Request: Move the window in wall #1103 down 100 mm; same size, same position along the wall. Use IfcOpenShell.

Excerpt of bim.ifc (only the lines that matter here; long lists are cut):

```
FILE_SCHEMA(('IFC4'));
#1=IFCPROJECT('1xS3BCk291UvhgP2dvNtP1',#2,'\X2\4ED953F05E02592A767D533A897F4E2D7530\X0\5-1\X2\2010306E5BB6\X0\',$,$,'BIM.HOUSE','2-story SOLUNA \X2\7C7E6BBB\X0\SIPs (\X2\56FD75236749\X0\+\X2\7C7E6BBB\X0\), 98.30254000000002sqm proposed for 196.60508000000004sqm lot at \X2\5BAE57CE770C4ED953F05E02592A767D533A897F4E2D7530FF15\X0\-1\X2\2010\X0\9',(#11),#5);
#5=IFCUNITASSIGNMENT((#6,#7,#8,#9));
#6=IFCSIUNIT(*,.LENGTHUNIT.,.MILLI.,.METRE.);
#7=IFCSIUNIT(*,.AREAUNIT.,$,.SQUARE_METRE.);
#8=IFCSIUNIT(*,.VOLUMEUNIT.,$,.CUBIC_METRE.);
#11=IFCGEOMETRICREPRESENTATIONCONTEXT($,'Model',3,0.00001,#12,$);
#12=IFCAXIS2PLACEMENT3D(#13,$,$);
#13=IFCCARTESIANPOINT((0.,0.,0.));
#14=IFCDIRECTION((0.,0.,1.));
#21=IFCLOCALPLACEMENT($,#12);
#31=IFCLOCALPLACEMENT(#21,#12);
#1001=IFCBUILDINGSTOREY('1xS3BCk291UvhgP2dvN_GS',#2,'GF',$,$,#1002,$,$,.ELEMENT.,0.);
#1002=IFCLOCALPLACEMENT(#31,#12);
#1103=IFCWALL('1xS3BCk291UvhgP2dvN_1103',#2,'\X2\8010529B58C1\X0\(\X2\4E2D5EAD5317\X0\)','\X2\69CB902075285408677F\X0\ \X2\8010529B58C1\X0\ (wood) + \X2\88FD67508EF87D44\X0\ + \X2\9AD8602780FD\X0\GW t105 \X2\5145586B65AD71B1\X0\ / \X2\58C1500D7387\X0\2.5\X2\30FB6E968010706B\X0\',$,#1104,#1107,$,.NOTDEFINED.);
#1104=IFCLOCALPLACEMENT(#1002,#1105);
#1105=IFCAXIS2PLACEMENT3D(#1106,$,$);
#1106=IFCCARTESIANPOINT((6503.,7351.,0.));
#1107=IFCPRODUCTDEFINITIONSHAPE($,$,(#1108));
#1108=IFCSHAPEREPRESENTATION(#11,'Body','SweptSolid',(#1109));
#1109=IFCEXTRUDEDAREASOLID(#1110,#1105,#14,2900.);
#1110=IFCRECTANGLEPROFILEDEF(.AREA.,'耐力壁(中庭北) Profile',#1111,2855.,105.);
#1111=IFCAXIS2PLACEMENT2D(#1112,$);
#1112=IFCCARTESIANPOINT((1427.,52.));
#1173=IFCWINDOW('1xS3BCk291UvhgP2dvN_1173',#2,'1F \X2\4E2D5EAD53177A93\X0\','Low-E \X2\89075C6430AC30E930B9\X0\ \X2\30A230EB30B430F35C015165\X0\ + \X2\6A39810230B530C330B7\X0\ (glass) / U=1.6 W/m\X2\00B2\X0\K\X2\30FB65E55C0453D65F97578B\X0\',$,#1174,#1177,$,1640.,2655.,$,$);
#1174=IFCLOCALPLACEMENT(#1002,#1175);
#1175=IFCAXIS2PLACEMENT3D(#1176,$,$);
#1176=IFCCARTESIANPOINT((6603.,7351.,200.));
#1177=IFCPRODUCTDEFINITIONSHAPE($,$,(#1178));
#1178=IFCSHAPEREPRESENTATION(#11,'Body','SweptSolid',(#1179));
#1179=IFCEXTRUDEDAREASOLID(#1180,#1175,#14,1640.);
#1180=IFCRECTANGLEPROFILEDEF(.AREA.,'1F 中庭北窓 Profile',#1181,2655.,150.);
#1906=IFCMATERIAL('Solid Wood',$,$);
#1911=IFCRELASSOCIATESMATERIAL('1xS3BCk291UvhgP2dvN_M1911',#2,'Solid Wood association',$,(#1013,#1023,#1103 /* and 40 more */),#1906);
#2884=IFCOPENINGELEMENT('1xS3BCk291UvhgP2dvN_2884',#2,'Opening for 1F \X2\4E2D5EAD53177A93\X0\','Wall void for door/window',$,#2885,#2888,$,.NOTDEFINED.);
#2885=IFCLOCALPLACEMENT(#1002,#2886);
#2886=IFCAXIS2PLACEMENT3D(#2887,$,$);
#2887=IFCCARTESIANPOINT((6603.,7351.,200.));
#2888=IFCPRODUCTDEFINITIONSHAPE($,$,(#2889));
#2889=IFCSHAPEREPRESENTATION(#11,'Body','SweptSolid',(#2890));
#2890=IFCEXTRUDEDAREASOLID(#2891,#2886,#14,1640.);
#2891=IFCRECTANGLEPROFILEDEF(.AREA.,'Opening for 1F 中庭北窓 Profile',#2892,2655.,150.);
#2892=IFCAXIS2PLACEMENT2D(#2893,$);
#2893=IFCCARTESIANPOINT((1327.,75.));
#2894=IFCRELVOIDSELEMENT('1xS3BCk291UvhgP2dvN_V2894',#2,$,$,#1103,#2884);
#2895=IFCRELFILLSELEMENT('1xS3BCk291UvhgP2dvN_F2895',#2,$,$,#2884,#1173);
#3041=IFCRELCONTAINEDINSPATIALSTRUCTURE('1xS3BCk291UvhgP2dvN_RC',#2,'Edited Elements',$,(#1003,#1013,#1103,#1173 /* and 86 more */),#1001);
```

```python
import numpy as np
import ifcopenshell
import ifcopenshell.api.geometry
import ifcopenshell.util.placement
import ifcopenshell.util.unit

model = ifcopenshell.open("bim.ifc")
unit_scale = ifcopenshell.util.unit.calculate_unit_scale(model)

window = model.by_guid("1xS3BCk291UvhgP2dvN_1173")
opening = window.FillsVoids[0].RelatingOpeningElement
dz = -100.0

shift = np.array([0.0, 0.0, dz])
# The window is not placed relative to its opening, so move both.
for product in (opening, window):
    matrix = ifcopenshell.util.placement.get_local_placement(product.ObjectPlacement)
    matrix[:3, 3] += shift
    ifcopenshell.api.geometry.edit_object_placement(model, product=product, matrix=matrix, is_si=False)

print(f"moved by {dz * unit_scale:+.3f} m")

model.write("bim_v2.ifc")
```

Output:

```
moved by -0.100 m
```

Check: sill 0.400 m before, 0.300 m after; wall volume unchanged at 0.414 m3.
